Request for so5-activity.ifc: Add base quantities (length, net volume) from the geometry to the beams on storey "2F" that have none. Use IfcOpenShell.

First a look at what the model holds.

```python
import ifcopenshell
import ifcopenshell.util.element
import ifcopenshell.util.unit

model = ifcopenshell.open("so5-activity.ifc")
print(model.schema)
for unit_type in ("LENGTHUNIT", "AREAUNIT", "VOLUMEUNIT"):
    print(unit_type, ifcopenshell.util.unit.calculate_unit_scale(model, unit_type))
storey = next(s for s in model.by_type("IfcBuildingStorey") if s.Name == "2F")
beams = [e for e in ifcopenshell.util.element.get_decomposition(storey) if e.is_a("IfcBeam")]
for e in sorted(beams, key=lambda e: e.id()):
    print(e.id(), e.is_a(), e.Name, list(ifcopenshell.util.element.get_psets(e, qtos_only=True)), sep=" | ")
```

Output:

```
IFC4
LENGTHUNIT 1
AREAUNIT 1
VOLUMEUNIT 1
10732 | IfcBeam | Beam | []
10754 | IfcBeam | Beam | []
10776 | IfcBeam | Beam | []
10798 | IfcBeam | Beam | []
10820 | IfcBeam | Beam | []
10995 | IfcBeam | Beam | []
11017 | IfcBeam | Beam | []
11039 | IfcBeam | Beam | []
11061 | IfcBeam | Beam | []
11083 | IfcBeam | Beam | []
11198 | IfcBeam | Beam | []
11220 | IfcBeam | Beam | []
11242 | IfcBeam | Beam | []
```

```python
import ifcopenshell
import ifcopenshell.api.pset
import ifcopenshell.geom
import ifcopenshell.util.element
import ifcopenshell.util.shape
import ifcopenshell.util.unit

model = ifcopenshell.open("so5-activity.ifc")
unit_scale = ifcopenshell.util.unit.calculate_unit_scale(model)
volume_scale = ifcopenshell.util.unit.calculate_unit_scale(model, "VOLUMEUNIT")
settings = ifcopenshell.geom.settings()

storey = next(s for s in model.by_type("IfcBuildingStorey") if s.Name == "2F")
beams = [e for e in ifcopenshell.util.element.get_decomposition(storey) if e.is_a("IfcBeam")]

for e in sorted(beams, key=lambda e: e.id()):
    if ifcopenshell.util.element.get_psets(e, qtos_only=True, should_inherit=False):
        continue
    # Geometry comes back in metres, in the element's own axes.
    shape = ifcopenshell.geom.create_shape(settings, e)
    values = {
        "Length": ifcopenshell.util.shape.get_max_xyz(shape.geometry) / unit_scale,
        "NetVolume": ifcopenshell.util.shape.get_volume(shape.geometry) / volume_scale,
    }
    qto = ifcopenshell.api.pset.add_qto(model, product=e, name="Qto_BeamBaseQuantities")
    ifcopenshell.api.pset.edit_qto(model, qto=qto, properties=values)
    print(e.id(), {k: round(v, 3) for k, v in values.items()})

model.write("so5-activity_rev.ifc")
```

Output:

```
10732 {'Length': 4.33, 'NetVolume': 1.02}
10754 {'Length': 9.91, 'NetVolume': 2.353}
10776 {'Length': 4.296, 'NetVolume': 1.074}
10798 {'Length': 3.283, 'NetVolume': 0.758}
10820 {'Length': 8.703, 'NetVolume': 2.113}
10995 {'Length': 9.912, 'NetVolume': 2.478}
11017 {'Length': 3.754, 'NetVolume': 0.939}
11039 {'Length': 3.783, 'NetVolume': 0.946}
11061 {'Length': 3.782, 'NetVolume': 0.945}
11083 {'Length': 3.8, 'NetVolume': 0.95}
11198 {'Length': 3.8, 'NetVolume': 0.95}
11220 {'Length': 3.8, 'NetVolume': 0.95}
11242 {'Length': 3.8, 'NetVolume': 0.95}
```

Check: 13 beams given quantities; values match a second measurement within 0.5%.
